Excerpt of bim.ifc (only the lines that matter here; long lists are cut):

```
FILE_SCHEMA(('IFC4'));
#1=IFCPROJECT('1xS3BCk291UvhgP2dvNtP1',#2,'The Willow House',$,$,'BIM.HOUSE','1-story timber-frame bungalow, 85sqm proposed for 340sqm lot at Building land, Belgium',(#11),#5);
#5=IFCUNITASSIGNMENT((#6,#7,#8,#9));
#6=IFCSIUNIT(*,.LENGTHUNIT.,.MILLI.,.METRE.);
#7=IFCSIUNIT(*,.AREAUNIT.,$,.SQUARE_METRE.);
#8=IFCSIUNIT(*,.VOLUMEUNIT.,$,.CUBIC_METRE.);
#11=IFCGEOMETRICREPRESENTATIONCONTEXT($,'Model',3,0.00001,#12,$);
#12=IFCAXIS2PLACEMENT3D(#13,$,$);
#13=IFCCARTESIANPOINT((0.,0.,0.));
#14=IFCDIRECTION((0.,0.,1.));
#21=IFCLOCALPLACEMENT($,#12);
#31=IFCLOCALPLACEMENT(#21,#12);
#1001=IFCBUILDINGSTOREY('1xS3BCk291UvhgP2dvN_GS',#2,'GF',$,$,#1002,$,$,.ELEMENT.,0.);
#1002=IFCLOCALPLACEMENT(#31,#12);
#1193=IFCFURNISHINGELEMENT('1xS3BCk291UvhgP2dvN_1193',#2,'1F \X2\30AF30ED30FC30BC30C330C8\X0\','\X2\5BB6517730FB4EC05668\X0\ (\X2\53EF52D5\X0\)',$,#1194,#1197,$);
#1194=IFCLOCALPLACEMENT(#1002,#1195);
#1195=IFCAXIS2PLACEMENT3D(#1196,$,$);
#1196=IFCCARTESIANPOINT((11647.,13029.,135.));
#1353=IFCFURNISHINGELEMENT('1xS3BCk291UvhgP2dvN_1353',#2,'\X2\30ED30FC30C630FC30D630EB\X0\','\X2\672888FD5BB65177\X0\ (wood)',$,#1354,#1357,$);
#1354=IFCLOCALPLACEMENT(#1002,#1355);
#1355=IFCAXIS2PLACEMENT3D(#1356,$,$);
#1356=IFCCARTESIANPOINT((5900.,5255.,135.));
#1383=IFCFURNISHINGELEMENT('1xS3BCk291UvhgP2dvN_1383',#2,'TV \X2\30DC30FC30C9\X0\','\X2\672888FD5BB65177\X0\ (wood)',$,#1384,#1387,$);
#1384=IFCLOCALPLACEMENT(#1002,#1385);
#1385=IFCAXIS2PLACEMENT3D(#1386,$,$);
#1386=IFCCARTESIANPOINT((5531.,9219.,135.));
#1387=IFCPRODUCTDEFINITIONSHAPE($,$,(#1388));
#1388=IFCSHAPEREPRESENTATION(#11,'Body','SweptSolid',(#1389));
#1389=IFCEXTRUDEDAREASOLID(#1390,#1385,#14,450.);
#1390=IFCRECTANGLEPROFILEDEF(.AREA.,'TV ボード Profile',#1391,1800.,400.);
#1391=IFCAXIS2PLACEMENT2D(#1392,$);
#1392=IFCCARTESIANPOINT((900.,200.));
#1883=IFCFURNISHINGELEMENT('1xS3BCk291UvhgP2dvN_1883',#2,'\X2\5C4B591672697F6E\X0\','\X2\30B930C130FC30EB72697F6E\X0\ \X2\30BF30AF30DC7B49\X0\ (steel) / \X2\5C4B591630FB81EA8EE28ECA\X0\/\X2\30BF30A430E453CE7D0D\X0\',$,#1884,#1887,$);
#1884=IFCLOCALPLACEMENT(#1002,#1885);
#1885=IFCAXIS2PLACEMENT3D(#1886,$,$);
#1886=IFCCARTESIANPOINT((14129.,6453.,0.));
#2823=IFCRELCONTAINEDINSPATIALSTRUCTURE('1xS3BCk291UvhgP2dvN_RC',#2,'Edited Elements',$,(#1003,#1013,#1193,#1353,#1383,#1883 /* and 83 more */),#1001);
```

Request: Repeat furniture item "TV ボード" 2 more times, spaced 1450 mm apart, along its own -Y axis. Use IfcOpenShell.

```python
import ifcopenshell
import ifcopenshell.api.geometry
import ifcopenshell.api.root
import ifcopenshell.util.element
import ifcopenshell.util.placement

model = ifcopenshell.open("bim.ifc")


def reuse_history(source, copy):
    """copy_class also copies each property set's owner history, people and application; keep the originals."""
    for rel in copy.IsDefinedBy:
        if rel.is_a("IfcRelDefinesByProperties") and (history := rel.RelatingPropertyDefinition.OwnerHistory):
            rel.RelatingPropertyDefinition.OwnerHistory = source.OwnerHistory
            ifcopenshell.util.element.remove_deep2(model, history)


source = model.by_guid("1xS3BCk291UvhgP2dvN_1383")
base = ifcopenshell.util.placement.get_local_placement(source.ObjectPlacement)
step = -base[:3, 1] * 1450.0

for i in range(1, 3):
    copy = ifcopenshell.api.root.copy_class(model, product=source)
    copy.Representation = ifcopenshell.util.element.copy_deep(
        model, source.Representation, exclude=["IfcGeometricRepresentationContext", "IfcRepresentationMap"]
    )
    reuse_history(source, copy)
    matrix = base.copy()
    matrix[:3, 3] += i * step
    print("added at", matrix[:3, 3].round(3) + 0.0)
    ifcopenshell.api.geometry.edit_object_placement(model, product=copy, matrix=matrix, is_si=False)

model.write("bim_rev.ifc")
```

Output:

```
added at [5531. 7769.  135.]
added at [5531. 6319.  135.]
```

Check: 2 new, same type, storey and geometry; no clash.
